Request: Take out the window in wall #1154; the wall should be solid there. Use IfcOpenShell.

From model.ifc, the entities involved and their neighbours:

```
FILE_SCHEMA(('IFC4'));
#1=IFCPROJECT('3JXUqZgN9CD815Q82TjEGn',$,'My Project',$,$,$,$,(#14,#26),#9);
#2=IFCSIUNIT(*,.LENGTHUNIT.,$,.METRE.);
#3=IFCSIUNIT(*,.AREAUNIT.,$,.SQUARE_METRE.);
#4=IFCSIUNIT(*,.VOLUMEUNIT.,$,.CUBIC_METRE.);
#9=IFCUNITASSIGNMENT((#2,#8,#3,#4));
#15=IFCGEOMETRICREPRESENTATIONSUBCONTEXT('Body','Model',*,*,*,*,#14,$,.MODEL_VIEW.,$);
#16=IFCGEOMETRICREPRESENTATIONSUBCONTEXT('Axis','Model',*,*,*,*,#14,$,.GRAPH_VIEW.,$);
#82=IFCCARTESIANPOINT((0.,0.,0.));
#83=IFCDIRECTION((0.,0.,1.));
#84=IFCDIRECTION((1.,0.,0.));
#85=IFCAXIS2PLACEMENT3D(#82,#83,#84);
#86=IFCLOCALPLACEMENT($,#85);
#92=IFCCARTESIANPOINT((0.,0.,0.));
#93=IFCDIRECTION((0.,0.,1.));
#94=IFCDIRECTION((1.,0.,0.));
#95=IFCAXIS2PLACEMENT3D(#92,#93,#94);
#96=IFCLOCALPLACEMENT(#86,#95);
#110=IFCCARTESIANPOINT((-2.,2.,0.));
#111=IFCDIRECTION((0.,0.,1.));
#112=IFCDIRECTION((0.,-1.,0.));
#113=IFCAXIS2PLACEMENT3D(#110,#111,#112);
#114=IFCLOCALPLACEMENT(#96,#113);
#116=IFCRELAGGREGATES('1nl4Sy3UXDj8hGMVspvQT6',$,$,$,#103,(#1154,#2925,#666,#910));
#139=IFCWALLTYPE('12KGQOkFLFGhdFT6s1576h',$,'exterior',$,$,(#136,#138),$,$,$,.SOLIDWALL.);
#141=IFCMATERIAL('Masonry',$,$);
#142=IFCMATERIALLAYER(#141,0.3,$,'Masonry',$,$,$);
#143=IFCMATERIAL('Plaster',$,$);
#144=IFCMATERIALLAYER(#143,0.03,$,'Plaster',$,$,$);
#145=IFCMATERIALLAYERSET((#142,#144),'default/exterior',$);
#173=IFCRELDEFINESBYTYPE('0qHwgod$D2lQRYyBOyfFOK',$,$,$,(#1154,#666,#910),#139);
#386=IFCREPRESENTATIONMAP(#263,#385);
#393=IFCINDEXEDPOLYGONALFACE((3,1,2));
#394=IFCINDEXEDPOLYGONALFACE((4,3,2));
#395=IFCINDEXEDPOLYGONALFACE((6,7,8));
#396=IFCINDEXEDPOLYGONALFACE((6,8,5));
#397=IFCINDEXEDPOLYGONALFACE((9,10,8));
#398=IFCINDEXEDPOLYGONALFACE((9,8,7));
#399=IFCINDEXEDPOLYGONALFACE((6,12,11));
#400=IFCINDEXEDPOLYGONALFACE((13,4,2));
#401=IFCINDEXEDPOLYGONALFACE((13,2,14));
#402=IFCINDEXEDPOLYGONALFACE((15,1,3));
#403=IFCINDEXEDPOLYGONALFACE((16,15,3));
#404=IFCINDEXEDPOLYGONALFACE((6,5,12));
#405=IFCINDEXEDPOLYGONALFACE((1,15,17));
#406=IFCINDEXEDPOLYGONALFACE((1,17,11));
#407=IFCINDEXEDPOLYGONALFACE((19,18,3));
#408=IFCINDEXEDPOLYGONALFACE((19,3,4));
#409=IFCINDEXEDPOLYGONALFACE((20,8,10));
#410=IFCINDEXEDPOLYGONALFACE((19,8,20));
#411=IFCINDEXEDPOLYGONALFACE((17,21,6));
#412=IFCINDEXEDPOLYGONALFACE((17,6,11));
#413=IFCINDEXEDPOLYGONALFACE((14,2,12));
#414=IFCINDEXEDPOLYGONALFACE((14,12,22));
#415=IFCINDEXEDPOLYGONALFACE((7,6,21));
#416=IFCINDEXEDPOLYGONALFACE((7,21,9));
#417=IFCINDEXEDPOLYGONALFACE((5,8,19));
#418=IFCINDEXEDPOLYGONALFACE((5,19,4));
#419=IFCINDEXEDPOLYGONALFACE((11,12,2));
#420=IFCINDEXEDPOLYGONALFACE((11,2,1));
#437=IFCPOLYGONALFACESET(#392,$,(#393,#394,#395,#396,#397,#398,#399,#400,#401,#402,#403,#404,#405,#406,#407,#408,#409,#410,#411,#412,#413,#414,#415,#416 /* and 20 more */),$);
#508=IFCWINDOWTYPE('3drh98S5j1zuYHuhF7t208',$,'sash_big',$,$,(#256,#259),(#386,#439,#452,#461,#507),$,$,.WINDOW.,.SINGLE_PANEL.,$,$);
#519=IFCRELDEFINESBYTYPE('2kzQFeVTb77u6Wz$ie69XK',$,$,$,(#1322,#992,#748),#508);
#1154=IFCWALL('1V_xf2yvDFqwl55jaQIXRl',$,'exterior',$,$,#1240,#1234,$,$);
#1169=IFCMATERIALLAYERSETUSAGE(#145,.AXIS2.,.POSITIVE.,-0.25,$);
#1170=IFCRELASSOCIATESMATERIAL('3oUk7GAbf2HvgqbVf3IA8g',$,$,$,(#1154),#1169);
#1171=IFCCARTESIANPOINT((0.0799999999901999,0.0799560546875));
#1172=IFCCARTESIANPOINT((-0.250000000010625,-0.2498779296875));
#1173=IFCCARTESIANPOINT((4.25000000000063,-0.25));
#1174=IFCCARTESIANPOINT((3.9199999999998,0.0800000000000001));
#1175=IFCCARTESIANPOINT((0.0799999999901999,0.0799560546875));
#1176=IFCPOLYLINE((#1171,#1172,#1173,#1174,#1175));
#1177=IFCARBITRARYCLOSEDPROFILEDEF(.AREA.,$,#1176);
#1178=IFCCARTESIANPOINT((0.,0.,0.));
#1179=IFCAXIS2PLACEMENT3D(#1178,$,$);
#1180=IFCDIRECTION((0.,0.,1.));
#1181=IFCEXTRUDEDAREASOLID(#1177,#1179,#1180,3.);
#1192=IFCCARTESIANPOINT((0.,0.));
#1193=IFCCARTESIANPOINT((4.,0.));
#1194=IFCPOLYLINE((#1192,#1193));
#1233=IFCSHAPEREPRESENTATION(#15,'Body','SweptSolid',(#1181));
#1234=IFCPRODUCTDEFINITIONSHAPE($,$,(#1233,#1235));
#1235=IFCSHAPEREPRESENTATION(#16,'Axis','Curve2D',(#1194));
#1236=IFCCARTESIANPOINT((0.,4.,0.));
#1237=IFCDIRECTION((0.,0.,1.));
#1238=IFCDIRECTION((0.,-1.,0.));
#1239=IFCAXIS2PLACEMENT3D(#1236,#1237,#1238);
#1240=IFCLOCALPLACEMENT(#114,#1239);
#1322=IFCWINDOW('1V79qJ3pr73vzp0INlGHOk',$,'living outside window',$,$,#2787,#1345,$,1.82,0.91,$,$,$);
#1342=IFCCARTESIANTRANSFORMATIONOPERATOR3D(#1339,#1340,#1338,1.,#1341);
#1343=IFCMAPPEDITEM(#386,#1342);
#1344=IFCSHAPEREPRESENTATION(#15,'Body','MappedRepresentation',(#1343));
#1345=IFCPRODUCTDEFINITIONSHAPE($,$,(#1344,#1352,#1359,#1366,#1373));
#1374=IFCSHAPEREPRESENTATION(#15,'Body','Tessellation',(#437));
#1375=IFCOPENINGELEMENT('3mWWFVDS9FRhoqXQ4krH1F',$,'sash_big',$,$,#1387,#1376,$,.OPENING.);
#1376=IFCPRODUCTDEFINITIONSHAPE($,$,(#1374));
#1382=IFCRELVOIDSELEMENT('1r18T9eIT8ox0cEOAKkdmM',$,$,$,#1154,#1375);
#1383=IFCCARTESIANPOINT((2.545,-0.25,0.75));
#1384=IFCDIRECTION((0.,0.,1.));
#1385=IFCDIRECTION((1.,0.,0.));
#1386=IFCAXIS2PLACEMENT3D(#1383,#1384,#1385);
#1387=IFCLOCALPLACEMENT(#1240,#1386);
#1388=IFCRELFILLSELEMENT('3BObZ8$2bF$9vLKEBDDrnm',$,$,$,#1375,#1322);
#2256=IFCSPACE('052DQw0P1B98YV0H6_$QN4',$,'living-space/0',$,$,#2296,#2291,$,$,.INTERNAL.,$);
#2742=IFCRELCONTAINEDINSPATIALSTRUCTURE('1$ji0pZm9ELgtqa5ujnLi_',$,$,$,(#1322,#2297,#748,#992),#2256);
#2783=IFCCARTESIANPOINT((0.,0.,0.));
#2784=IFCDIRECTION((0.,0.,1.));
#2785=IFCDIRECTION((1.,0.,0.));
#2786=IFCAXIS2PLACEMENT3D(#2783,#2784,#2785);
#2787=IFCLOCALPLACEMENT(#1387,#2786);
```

```python
import ifcopenshell
import ifcopenshell.api.feature
import ifcopenshell.api.root
import ifcopenshell.geom
import ifcopenshell.util.shape

model = ifcopenshell.open("model.ifc")
settings = ifcopenshell.geom.settings()


def volume(element):
    """Net volume in cubic metres, openings subtracted."""
    shape = ifcopenshell.geom.create_shape(settings, element)
    return ifcopenshell.util.shape.get_volume(shape.geometry)


window = model.by_guid("1V79qJ3pr73vzp0INlGHOk")
opening = window.FillsVoids[0].RelatingOpeningElement
wall = opening.VoidsElements[0].RelatingBuildingElement
before = volume(wall)

ifcopenshell.api.root.remove_product(model, product=window)
ifcopenshell.api.feature.remove_feature(model, feature=opening)

after = volume(wall)

print(f"wall volume {before:.3f} -> {after:.3f} m3")

model.write("model_updated.ifc")
```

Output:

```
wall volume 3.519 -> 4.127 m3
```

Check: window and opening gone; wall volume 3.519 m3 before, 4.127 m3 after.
